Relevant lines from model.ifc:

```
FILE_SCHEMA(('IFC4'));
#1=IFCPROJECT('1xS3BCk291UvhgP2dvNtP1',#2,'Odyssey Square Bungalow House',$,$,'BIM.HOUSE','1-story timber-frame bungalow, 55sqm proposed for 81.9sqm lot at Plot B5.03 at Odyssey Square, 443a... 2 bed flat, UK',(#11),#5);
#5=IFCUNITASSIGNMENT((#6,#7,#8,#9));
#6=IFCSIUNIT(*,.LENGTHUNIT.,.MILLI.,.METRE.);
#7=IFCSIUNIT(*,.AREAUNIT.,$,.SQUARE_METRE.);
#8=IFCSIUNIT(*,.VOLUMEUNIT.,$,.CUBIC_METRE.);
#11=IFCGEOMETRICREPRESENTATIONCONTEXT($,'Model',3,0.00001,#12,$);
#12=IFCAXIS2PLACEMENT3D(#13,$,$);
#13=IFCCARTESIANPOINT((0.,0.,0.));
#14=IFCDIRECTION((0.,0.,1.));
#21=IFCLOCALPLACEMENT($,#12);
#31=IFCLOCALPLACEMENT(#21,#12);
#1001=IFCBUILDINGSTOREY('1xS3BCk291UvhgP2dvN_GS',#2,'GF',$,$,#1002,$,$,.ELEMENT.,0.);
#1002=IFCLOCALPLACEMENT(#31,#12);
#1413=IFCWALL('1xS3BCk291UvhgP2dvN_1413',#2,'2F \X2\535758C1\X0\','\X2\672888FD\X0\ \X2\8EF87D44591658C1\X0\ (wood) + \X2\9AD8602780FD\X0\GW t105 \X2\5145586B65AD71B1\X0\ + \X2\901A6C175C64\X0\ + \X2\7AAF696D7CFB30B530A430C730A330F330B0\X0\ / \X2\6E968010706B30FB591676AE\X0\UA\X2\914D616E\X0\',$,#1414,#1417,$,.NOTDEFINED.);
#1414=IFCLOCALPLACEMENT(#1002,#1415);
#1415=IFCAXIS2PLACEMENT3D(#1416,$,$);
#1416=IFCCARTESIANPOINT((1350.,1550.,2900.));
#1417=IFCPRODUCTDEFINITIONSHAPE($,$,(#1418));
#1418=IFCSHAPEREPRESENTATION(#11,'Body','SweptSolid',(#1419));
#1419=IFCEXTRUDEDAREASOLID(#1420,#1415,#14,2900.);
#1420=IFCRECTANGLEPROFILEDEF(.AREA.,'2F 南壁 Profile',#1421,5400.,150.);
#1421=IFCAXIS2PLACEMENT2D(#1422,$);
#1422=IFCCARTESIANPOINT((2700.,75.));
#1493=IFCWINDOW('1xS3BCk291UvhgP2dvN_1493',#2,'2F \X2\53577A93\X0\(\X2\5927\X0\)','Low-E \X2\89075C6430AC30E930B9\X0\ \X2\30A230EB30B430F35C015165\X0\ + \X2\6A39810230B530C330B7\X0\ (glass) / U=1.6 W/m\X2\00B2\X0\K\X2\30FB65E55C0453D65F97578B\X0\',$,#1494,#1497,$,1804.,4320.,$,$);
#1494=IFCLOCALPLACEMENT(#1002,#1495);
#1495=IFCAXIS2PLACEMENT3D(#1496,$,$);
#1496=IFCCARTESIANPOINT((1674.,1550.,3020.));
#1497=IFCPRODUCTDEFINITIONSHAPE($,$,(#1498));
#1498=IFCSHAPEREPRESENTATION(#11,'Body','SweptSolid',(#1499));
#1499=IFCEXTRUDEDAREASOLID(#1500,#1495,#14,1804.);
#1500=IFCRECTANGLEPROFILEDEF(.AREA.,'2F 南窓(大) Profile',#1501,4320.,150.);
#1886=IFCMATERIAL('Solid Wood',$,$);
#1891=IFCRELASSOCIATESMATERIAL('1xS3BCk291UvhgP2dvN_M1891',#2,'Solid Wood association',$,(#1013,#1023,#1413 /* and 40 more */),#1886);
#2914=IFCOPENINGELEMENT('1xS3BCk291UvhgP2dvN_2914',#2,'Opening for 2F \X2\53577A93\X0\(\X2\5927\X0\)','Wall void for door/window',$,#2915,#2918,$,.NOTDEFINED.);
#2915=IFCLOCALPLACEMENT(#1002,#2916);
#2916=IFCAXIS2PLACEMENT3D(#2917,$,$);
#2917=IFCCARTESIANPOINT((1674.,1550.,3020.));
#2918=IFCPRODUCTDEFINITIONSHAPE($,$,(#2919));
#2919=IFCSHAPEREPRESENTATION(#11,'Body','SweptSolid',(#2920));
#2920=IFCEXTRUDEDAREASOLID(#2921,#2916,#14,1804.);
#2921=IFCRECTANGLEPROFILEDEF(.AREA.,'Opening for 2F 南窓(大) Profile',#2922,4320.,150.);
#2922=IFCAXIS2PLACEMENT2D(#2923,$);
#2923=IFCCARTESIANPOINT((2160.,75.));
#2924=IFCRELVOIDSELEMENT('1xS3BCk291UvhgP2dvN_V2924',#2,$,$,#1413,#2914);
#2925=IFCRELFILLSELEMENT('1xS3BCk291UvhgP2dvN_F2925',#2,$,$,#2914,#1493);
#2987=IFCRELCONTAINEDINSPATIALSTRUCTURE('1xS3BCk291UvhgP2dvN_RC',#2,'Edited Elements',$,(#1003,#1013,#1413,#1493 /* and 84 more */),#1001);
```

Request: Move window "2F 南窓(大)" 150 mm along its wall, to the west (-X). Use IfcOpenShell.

```python
import ifcopenshell
import ifcopenshell.api.geometry
import ifcopenshell.util.placement
import ifcopenshell.util.unit

model = ifcopenshell.open("model.ifc")
unit_scale = ifcopenshell.util.unit.calculate_unit_scale(model)

window = model.by_guid("1xS3BCk291UvhgP2dvN_1493")
opening = window.FillsVoids[0].RelatingOpeningElement
wall = opening.VoidsElements[0].RelatingBuildingElement

wall_matrix = ifcopenshell.util.placement.get_local_placement(wall.ObjectPlacement)
shift = wall_matrix[:3, 0] * -0.15 / unit_scale
before = ifcopenshell.util.placement.get_local_placement(window.ObjectPlacement)[:3, 3].copy()

# The window is not placed relative to its opening, so move both.
for product in (opening, window):
    matrix = ifcopenshell.util.placement.get_local_placement(product.ObjectPlacement)
    matrix[:3, 3] += shift
    ifcopenshell.api.geometry.edit_object_placement(model, product=product, matrix=matrix, is_si=False)

after = ifcopenshell.util.placement.get_local_placement(window.ObjectPlacement)[:3, 3]
print("window moved by", (after - before).round(3) + 0.0)

model.write("model_rev.ifc")
```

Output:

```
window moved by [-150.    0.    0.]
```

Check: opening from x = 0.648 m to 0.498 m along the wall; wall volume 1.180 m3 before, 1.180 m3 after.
